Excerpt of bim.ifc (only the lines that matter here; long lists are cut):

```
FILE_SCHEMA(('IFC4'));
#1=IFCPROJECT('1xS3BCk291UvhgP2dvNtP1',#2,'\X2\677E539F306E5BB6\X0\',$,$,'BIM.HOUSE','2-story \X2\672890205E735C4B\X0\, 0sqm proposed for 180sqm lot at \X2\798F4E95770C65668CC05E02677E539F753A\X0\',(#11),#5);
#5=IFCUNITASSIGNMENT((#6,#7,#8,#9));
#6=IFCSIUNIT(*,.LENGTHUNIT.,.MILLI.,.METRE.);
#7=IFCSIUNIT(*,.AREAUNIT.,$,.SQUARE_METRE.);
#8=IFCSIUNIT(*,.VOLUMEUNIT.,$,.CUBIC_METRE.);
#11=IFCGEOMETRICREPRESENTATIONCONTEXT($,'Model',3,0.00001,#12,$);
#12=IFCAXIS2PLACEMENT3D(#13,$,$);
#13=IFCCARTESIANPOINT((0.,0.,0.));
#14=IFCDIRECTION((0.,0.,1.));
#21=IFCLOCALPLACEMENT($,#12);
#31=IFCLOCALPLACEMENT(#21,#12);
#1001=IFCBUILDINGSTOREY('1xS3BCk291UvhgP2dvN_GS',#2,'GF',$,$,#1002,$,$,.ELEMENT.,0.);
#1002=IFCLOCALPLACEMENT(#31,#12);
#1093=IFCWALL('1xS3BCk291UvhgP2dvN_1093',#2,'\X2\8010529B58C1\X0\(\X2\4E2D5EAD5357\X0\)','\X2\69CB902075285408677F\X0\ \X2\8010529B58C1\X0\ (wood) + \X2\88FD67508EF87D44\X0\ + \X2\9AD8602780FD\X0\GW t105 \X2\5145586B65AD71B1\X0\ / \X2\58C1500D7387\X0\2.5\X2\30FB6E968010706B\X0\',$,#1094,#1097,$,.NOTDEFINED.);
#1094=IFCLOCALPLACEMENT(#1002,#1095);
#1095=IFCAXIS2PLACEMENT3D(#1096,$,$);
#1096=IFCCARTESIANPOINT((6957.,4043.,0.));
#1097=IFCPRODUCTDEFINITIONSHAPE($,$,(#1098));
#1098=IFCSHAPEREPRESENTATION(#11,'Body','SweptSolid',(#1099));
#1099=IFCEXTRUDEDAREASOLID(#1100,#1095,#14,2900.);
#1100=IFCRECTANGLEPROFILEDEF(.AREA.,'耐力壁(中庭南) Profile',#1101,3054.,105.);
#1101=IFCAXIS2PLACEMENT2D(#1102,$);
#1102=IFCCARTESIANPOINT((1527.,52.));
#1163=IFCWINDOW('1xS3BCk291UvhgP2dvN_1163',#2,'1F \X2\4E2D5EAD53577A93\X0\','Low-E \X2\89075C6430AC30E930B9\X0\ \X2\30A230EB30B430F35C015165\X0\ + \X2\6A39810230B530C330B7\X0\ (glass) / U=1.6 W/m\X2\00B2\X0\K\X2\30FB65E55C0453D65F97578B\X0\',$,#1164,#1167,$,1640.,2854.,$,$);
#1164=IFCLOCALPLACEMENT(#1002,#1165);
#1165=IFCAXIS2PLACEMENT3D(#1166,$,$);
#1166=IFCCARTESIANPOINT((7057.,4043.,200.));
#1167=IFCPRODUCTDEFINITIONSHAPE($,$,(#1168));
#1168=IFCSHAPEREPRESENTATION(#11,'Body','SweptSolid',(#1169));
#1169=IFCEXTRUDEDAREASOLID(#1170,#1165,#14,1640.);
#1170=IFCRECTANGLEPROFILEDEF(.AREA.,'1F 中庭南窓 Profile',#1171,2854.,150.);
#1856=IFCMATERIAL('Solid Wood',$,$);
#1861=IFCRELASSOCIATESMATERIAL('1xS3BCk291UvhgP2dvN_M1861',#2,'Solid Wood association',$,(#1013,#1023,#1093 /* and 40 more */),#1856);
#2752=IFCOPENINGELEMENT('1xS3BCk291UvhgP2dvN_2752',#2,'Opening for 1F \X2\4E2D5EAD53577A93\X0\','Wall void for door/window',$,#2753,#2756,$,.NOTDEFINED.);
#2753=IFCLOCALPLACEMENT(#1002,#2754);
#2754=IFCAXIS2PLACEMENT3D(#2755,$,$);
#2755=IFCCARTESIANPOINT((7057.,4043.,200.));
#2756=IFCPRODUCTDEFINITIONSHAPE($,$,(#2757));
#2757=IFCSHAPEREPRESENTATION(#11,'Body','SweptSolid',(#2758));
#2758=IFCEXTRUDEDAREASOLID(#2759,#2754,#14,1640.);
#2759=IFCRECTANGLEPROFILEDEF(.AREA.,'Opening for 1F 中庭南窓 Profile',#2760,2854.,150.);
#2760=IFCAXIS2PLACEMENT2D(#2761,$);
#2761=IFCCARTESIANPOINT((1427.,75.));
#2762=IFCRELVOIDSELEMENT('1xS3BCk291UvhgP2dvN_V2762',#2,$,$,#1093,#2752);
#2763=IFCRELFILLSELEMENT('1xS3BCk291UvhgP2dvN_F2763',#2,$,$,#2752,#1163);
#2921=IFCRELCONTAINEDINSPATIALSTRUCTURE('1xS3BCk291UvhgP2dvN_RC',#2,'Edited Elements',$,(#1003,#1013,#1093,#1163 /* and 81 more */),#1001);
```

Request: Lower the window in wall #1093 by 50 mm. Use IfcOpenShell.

```python
import numpy as np
import ifcopenshell
import ifcopenshell.api.geometry
import ifcopenshell.util.placement
import ifcopenshell.util.unit

model = ifcopenshell.open("bim.ifc")
unit_scale = ifcopenshell.util.unit.calculate_unit_scale(model)

window = model.by_guid("1xS3BCk291UvhgP2dvN_1163")
opening = window.FillsVoids[0].RelatingOpeningElement
dz = -0.05 / unit_scale

shift = np.array([0.0, 0.0, dz])
# The window is not placed relative to its opening, so move both.
for product in (opening, window):
    matrix = ifcopenshell.util.placement.get_local_placement(product.ObjectPlacement)
    matrix[:3, 3] += shift
    ifcopenshell.api.geometry.edit_object_placement(model, product=product, matrix=matrix, is_si=False)

print(f"moved by {dz * unit_scale:+.3f} m")

model.write("bim_v2.ifc")
```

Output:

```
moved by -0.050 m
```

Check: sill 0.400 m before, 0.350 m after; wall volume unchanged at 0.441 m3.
